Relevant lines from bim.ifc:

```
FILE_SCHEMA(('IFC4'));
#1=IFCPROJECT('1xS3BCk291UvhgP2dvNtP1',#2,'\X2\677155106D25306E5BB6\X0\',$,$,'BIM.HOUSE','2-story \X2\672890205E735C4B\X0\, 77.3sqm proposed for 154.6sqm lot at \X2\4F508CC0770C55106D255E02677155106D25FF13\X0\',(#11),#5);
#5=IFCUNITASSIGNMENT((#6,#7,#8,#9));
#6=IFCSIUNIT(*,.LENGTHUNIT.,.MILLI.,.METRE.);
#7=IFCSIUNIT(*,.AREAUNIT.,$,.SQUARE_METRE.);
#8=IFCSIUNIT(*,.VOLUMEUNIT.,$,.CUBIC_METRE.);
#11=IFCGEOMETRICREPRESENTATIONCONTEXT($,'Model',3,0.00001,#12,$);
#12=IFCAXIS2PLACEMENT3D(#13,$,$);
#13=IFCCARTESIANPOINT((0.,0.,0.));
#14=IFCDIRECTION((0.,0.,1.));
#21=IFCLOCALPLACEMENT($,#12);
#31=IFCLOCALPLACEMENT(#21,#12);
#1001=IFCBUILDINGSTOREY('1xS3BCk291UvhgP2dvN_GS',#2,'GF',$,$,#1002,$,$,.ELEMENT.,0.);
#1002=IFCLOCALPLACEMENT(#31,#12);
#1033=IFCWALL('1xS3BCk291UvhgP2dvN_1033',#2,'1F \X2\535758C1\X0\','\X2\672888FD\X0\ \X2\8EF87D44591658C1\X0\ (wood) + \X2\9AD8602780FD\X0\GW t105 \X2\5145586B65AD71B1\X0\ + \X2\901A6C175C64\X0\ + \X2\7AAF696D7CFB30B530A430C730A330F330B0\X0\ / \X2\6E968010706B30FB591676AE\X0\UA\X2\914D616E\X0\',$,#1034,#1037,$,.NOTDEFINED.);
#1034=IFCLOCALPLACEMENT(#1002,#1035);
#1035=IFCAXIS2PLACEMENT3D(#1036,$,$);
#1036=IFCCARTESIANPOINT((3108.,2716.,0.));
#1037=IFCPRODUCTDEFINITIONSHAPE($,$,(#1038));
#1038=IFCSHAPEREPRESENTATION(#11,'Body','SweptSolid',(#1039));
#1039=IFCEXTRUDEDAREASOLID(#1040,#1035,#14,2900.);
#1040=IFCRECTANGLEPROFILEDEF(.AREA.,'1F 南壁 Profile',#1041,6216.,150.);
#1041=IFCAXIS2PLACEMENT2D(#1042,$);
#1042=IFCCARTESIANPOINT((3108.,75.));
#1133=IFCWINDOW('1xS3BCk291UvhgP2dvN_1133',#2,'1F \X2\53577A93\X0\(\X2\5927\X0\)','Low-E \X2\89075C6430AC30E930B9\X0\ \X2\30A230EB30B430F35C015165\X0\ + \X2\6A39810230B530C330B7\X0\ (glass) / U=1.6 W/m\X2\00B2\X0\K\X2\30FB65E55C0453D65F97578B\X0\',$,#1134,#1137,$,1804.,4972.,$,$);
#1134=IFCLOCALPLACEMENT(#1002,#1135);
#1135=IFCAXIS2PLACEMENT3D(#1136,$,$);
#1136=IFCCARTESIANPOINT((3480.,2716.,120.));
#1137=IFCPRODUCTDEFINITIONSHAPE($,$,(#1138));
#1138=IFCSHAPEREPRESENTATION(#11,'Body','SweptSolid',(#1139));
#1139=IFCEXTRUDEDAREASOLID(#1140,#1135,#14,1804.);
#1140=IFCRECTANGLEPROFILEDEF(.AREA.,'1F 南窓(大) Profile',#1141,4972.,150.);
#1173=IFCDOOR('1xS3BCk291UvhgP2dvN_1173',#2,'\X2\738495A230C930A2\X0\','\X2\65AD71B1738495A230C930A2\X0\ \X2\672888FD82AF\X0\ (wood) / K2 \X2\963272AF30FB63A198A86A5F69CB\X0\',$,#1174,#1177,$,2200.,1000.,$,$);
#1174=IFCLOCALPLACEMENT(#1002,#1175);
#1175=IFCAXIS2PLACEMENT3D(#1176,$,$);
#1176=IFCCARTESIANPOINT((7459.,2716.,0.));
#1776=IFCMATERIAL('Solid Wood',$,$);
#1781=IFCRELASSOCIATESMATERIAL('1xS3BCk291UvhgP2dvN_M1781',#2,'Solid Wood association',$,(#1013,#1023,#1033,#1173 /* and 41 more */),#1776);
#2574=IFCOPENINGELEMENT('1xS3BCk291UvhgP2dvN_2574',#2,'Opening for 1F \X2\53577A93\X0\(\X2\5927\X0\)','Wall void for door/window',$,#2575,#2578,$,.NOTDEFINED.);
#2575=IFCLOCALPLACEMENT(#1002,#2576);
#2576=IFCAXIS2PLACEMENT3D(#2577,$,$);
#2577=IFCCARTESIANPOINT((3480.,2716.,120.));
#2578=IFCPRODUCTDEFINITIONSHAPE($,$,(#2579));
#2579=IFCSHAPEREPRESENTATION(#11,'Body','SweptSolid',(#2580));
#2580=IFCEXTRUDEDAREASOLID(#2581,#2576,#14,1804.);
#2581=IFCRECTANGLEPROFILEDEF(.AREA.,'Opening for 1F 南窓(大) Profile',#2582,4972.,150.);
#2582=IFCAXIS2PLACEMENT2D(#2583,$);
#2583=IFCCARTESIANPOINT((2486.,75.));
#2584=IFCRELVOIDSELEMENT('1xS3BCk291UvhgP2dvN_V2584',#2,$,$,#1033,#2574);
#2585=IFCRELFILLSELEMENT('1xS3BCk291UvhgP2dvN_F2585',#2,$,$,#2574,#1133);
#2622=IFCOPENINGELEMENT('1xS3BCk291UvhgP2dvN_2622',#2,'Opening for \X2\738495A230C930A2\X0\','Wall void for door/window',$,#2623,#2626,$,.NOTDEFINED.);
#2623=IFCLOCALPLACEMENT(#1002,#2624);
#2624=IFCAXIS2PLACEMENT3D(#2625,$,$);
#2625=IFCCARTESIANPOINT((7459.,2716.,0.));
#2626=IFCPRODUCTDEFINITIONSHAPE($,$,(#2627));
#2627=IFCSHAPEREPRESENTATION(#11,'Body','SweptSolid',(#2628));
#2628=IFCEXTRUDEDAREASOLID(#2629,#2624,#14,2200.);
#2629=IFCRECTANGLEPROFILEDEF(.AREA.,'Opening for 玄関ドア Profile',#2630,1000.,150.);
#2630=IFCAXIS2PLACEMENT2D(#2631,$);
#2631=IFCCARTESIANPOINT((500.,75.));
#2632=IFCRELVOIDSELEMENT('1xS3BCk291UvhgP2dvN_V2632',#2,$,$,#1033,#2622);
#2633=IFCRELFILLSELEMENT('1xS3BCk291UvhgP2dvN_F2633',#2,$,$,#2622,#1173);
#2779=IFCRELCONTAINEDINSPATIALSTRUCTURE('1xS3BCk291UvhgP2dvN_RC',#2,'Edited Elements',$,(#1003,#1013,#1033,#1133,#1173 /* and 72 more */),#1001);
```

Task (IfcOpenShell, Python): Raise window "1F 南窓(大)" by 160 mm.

```python
import numpy as np
import ifcopenshell
import ifcopenshell.api.geometry
import ifcopenshell.util.placement
import ifcopenshell.util.unit

model = ifcopenshell.open("bim.ifc")
unit_scale = ifcopenshell.util.unit.calculate_unit_scale(model)

window = model.by_id(1133)
opening = window.FillsVoids[0].RelatingOpeningElement
dz = 0.16 / unit_scale

shift = np.array([0.0, 0.0, dz])
# The window is not placed relative to its opening, so move both.
for product in (opening, window):
    matrix = ifcopenshell.util.placement.get_local_placement(product.ObjectPlacement)
    matrix[:3, 3] += shift
    ifcopenshell.api.geometry.edit_object_placement(model, product=product, matrix=matrix, is_si=False)

print(f"moved by {dz * unit_scale:+.3f} m")

model.write("bim_edited.ifc")
```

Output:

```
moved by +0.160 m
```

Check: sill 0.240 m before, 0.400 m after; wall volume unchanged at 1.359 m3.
